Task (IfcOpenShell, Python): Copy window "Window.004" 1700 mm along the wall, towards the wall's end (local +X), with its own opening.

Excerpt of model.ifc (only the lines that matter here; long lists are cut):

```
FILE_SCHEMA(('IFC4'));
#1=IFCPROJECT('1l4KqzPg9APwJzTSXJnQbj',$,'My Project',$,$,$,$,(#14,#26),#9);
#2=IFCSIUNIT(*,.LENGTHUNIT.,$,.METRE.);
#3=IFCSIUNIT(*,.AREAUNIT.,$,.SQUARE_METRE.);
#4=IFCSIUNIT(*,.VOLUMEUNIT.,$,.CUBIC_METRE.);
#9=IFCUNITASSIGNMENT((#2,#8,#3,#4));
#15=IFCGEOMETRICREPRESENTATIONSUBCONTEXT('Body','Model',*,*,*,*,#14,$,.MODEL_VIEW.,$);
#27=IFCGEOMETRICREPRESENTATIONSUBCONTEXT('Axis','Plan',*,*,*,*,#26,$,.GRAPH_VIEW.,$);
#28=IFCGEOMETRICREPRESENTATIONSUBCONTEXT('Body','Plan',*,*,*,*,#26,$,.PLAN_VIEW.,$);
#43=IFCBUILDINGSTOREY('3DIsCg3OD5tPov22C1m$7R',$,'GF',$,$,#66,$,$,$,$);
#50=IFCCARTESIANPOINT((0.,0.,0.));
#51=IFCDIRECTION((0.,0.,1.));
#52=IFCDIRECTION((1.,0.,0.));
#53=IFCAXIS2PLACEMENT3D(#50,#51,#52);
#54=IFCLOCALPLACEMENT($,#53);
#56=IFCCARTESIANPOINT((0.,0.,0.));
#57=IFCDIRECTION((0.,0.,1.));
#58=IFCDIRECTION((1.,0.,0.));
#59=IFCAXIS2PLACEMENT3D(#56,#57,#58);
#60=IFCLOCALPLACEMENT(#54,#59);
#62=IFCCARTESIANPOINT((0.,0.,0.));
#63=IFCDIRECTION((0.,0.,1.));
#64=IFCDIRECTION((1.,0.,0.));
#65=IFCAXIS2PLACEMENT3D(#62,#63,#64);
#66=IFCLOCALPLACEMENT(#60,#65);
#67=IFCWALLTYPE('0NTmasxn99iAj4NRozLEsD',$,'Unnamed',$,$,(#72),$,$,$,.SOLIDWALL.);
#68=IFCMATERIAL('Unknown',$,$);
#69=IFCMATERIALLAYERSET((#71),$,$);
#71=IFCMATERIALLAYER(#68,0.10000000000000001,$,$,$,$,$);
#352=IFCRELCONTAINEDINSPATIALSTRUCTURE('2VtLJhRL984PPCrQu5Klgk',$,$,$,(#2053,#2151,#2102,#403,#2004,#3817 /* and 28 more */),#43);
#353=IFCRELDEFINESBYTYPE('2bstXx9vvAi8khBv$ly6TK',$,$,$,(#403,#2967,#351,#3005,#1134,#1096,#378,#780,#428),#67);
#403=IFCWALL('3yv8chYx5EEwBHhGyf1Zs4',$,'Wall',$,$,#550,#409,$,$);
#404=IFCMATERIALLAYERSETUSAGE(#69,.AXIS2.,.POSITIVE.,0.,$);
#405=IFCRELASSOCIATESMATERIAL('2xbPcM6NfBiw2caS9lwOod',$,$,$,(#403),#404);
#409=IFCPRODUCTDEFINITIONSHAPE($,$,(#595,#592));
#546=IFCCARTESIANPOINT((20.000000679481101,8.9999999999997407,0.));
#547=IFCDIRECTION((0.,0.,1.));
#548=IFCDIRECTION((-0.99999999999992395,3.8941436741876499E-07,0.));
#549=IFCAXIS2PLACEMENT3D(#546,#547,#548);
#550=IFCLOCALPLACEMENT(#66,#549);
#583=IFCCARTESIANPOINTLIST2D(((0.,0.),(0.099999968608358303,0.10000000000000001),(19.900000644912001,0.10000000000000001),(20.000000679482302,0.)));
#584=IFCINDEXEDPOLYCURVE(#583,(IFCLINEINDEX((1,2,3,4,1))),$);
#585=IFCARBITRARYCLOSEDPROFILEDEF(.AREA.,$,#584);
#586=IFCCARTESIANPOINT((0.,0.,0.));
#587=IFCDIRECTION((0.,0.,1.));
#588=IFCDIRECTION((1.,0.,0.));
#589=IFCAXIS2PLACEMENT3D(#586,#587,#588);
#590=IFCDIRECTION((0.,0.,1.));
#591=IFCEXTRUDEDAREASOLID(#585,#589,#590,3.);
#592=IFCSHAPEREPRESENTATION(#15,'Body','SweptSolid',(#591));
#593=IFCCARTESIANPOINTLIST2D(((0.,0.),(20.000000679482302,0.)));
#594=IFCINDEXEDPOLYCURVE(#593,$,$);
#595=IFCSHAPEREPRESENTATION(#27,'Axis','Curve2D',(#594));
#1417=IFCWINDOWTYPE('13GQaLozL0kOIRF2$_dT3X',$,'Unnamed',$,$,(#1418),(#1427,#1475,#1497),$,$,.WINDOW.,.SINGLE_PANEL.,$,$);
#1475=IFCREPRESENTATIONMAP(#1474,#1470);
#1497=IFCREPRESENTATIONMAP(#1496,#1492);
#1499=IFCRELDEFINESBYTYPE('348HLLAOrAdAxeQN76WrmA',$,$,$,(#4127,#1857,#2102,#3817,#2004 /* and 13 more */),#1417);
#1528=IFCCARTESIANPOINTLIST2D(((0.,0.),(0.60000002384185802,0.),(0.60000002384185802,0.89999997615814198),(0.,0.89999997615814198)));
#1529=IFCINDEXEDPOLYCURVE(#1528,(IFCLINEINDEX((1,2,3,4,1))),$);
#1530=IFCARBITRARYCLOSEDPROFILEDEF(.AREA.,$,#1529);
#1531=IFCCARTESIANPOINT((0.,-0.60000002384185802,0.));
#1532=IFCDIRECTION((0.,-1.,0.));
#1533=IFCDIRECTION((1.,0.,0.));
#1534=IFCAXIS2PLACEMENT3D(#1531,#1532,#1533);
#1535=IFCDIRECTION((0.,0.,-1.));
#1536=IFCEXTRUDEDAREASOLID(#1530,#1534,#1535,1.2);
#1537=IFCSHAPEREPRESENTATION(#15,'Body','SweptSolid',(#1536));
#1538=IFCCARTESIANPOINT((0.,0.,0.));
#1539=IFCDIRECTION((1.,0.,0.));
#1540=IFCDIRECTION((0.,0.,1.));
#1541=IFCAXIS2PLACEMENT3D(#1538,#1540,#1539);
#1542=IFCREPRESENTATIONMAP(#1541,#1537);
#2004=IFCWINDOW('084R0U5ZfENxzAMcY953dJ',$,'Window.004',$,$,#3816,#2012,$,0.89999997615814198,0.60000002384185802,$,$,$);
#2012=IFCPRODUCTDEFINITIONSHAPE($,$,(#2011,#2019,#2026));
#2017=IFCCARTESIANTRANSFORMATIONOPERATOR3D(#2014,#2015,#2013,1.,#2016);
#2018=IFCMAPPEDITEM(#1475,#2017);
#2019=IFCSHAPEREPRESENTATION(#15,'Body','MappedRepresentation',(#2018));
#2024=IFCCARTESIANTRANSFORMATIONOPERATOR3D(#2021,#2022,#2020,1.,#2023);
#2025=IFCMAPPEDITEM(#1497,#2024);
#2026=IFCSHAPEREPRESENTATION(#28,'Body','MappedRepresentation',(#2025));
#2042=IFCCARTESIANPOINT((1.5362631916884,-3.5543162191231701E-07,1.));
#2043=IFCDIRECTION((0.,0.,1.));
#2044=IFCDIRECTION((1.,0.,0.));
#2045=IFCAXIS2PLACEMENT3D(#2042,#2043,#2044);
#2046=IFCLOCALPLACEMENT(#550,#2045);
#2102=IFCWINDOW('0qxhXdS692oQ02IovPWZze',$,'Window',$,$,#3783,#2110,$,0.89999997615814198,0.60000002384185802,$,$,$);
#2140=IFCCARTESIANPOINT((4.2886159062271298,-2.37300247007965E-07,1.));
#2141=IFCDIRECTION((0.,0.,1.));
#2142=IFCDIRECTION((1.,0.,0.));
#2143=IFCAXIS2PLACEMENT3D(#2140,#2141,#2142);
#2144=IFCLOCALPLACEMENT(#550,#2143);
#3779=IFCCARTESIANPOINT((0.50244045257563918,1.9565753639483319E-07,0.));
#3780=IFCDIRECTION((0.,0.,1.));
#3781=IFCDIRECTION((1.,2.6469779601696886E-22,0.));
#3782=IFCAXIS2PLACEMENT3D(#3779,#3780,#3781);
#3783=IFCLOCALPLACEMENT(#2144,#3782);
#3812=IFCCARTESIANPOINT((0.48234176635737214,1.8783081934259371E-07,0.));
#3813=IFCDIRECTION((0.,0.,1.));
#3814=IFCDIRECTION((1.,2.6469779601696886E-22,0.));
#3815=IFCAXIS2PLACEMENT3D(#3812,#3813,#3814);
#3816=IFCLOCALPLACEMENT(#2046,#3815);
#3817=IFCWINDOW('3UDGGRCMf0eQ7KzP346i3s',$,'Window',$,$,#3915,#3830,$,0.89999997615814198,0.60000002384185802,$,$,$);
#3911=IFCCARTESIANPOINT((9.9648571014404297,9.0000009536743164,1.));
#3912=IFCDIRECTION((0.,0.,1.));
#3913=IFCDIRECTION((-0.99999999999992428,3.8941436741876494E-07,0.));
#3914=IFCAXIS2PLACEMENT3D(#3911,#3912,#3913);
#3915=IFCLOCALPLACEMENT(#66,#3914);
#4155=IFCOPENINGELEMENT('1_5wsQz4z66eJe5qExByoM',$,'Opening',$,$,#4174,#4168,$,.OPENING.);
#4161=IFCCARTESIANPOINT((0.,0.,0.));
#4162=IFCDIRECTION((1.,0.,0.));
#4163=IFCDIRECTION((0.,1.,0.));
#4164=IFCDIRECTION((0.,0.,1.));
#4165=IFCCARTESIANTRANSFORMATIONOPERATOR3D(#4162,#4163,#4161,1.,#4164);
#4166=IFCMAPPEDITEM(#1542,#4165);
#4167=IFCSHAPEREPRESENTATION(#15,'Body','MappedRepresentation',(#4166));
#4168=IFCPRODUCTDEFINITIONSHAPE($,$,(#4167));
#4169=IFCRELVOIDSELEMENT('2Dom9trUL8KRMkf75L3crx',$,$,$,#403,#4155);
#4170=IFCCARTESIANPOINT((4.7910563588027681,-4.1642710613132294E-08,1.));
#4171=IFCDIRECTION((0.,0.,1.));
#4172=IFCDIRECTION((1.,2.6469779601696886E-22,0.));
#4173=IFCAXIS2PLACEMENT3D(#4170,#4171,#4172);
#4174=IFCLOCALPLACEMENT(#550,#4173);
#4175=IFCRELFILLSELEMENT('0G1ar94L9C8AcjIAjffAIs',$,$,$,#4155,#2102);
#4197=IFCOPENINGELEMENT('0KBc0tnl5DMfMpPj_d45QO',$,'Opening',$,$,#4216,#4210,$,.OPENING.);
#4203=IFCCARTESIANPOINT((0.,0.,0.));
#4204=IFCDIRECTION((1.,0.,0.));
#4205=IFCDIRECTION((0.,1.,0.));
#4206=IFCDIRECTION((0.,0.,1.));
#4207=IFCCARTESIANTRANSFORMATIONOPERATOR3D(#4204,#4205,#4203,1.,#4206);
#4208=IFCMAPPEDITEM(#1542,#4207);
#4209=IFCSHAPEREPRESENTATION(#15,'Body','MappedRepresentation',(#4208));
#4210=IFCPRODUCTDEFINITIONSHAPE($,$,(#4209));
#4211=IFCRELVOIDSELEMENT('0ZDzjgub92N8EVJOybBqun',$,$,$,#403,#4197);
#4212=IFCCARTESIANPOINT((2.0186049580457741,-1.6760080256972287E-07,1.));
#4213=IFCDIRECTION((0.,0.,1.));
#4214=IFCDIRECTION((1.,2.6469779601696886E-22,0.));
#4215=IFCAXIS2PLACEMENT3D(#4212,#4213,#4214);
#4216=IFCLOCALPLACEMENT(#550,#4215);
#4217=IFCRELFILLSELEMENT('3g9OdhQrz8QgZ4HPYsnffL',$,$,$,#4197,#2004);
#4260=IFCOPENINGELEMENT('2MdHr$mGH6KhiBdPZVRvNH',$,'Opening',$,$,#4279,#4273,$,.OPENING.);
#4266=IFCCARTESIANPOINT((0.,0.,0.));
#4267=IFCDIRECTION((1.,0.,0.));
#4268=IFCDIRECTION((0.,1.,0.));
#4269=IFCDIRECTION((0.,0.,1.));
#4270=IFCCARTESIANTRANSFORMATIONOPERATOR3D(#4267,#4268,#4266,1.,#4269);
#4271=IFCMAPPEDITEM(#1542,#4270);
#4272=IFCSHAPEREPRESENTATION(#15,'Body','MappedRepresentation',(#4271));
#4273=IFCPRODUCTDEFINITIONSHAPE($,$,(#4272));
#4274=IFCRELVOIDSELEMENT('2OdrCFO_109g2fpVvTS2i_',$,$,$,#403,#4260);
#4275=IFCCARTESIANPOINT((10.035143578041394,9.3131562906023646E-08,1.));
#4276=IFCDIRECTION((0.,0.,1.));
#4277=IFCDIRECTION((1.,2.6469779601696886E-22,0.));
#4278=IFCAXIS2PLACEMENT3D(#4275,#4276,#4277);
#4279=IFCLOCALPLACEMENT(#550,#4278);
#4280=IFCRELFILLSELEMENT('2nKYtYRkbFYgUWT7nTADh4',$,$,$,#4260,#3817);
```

```python
import ifcopenshell
import ifcopenshell.api.feature
import ifcopenshell.api.geometry
import ifcopenshell.api.root
import ifcopenshell.geom
import ifcopenshell.util.element
import ifcopenshell.util.placement
import ifcopenshell.util.shape

model = ifcopenshell.open("model.ifc")
settings = ifcopenshell.geom.settings()


def volume(element):
    """Net volume in cubic metres, openings subtracted."""
    shape = ifcopenshell.geom.create_shape(settings, element)
    return ifcopenshell.util.shape.get_volume(shape.geometry)


window = model.by_guid("084R0U5ZfENxzAMcY953dJ")
opening = window.FillsVoids[0].RelatingOpeningElement
wall = opening.VoidsElements[0].RelatingBuildingElement
before = volume(wall)
shift = ifcopenshell.util.placement.get_local_placement(wall.ObjectPlacement)[:3, 0] * 1.7

# copy_class copies the void relationship, type, container and properties, but no geometry.
new_opening = ifcopenshell.api.root.copy_class(model, product=opening)
new_opening.Representation = ifcopenshell.util.element.copy_deep(
    model, opening.Representation, exclude=["IfcGeometricRepresentationContext", "IfcRepresentationMap"]
)
new_window = ifcopenshell.api.root.copy_class(model, product=window)
new_window.Representation = ifcopenshell.util.element.copy_deep(
    model, window.Representation, exclude=["IfcGeometricRepresentationContext", "IfcRepresentationMap"]
)
ifcopenshell.api.feature.add_filling(model, opening=new_opening, element=new_window)

for old, new in ((opening, new_opening), (window, new_window)):
    matrix = ifcopenshell.util.placement.get_local_placement(old.ObjectPlacement)
    matrix[:3, 3] += shift
    ifcopenshell.api.geometry.edit_object_placement(model, product=new, matrix=matrix, is_si=False)

after = volume(wall)

print(f"wall volume {before:.3f} -> {after:.3f} m3")

model.write("model_edited.ifc")
```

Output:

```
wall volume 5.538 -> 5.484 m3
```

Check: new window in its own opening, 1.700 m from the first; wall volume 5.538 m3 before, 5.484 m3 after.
